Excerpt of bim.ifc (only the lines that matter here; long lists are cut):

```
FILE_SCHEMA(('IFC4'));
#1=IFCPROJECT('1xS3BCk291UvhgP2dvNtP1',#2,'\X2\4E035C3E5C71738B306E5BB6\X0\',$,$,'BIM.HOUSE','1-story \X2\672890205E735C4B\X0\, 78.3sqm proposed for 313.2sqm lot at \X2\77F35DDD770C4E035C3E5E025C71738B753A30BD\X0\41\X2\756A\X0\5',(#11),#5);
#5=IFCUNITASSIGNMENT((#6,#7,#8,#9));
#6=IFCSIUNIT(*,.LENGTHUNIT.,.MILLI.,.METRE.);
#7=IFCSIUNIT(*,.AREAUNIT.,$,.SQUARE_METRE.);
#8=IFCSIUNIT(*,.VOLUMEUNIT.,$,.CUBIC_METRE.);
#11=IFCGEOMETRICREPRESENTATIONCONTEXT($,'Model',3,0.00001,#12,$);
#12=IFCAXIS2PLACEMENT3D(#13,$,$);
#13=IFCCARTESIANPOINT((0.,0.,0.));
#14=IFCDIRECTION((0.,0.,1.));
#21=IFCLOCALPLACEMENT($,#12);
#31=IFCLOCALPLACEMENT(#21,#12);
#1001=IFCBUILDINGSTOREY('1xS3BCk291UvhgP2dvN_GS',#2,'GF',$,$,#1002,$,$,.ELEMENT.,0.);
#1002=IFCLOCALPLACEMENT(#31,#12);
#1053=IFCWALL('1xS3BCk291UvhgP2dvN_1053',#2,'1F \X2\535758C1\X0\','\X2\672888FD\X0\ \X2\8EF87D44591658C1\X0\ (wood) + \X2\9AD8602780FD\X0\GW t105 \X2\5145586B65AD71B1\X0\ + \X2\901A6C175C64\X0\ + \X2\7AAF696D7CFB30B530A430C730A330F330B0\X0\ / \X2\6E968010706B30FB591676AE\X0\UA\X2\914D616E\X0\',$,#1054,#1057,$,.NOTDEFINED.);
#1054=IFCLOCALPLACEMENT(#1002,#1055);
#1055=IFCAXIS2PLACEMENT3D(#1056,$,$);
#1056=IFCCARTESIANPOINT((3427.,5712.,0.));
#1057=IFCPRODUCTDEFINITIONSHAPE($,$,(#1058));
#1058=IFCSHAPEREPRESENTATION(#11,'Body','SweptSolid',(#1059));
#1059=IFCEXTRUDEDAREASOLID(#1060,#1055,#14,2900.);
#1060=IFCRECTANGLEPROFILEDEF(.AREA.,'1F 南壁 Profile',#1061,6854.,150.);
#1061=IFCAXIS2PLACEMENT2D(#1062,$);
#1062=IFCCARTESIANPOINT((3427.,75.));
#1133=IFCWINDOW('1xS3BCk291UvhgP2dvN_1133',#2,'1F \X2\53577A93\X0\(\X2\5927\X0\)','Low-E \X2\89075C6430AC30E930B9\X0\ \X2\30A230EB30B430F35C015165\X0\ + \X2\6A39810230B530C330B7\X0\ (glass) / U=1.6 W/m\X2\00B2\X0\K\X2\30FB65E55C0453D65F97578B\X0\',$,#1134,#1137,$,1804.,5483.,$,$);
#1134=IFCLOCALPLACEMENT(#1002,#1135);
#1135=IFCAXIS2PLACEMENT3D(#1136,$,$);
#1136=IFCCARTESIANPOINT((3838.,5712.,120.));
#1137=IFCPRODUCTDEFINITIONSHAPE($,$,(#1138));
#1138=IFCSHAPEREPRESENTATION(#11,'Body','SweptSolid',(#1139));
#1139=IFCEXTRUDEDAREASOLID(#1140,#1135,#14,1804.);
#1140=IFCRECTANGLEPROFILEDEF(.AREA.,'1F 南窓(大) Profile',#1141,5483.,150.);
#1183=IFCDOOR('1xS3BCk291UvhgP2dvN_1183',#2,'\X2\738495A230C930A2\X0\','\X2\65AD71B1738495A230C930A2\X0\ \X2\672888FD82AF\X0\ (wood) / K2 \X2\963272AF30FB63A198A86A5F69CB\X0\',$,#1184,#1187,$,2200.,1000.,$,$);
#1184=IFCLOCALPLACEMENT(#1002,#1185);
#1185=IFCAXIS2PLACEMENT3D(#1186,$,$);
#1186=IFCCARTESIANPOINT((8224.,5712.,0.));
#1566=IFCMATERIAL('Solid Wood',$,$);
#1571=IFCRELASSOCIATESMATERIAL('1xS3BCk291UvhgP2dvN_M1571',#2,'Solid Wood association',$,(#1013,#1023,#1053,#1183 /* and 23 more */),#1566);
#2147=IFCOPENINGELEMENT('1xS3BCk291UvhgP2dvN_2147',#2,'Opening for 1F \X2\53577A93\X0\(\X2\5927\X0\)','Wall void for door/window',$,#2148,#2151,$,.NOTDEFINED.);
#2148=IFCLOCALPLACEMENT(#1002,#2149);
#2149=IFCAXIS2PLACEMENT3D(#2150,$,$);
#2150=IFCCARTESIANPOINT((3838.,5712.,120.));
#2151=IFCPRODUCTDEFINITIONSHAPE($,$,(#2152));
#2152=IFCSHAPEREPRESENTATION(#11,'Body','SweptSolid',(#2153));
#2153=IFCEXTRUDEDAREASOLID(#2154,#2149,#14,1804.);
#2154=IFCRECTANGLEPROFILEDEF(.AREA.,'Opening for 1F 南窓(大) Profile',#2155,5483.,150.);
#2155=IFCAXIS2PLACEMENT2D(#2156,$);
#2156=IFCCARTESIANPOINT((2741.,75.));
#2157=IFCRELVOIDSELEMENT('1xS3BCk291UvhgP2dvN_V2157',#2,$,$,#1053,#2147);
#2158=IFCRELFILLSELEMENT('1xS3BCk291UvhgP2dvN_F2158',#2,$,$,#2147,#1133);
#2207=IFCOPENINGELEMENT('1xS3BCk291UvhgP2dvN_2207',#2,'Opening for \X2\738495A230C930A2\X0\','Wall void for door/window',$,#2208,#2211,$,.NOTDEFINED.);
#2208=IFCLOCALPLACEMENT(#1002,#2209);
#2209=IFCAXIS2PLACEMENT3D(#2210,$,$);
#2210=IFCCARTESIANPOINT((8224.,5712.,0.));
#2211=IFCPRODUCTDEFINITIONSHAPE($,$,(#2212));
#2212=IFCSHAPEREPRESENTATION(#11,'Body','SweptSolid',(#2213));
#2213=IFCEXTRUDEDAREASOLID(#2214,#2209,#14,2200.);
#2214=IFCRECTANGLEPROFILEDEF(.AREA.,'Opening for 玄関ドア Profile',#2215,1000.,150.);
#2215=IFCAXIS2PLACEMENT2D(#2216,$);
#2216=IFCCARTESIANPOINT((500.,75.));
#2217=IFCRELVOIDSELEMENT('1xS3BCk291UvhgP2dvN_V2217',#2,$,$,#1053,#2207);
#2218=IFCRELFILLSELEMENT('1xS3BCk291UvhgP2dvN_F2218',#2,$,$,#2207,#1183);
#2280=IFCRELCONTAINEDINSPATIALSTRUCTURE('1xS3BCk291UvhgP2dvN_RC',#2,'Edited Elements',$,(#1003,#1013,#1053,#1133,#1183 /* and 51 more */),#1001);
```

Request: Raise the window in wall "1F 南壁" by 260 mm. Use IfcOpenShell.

```python
import numpy as np
import ifcopenshell
import ifcopenshell.api.geometry
import ifcopenshell.util.placement
import ifcopenshell.util.unit

model = ifcopenshell.open("bim.ifc")
unit_scale = ifcopenshell.util.unit.calculate_unit_scale(model)

window = model.by_guid("1xS3BCk291UvhgP2dvN_1133")
opening = window.FillsVoids[0].RelatingOpeningElement
dz = 0.26 / unit_scale

shift = np.array([0.0, 0.0, dz])
# The window is not placed relative to its opening, so move both.
for product in (opening, window):
    matrix = ifcopenshell.util.placement.get_local_placement(product.ObjectPlacement)
    matrix[:3, 3] += shift
    ifcopenshell.api.geometry.edit_object_placement(model, product=product, matrix=matrix, is_si=False)

print(f"moved by {dz * unit_scale:+.3f} m")

model.write("bim_edited.ifc")
```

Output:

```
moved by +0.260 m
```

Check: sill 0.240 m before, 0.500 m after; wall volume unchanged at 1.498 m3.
